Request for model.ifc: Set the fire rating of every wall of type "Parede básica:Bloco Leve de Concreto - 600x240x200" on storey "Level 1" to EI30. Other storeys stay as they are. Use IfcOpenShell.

First a look at what the model holds.

```python
import ifcopenshell
import ifcopenshell.util.element

model = ifcopenshell.open("model.ifc")
print(model.schema)
storey = next(s for s in model.by_type("IfcBuildingStorey") if s.Name == "Level 1")
walls = [e for e in ifcopenshell.util.element.get_decomposition(storey) if e.is_a("IfcWall")]
seen = {}
for e in walls:
    element_type = ifcopenshell.util.element.get_type(e)
    key = (element_type.Name if element_type != e and element_type else None, ifcopenshell.util.element.get_pset(e, "Pset_WallCommon", "FireRating"))
    seen[key] = seen.get(key, 0) + 1
for (name, value), count in sorted(seen.items(), key=str):
    print(count, "x", name, "|", value)
```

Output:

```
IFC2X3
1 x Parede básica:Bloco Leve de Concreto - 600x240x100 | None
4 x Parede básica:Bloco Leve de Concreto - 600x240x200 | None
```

```python
import ifcopenshell
import ifcopenshell.api.pset
import ifcopenshell.util.element

model = ifcopenshell.open("model.ifc")

storey = next(s for s in model.by_type("IfcBuildingStorey") if s.Name == "Level 1")
walls = [e for e in ifcopenshell.util.element.get_decomposition(storey) if e.is_a("IfcWall")]

count = 0
for e in walls:
    element_type = ifcopenshell.util.element.get_type(e)
    if element_type in (None, e) or element_type.Name != "Parede básica:Bloco Leve de Concreto - 600x240x200":
        continue
    # add_pset returns the element's existing set when there is one.
    pset = ifcopenshell.api.pset.add_pset(model, product=e, name="Pset_WallCommon")
    ifcopenshell.api.pset.edit_pset(model, pset=pset, properties={"FireRating": "EI30"})
    count += 1

print(count, "walls updated")

model.write("model_edited.ifc")
```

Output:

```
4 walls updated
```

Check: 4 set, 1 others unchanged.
